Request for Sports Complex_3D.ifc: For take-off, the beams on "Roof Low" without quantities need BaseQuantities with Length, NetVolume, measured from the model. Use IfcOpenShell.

First a look at what the model holds.

```python
import ifcopenshell
import ifcopenshell.util.element
import ifcopenshell.util.unit

model = ifcopenshell.open("Sports Complex_3D.ifc")
print(model.schema)
for unit_type in ("LENGTHUNIT", "AREAUNIT", "VOLUMEUNIT"):
    print(unit_type, ifcopenshell.util.unit.calculate_unit_scale(model, unit_type))
storey = next(s for s in model.by_type("IfcBuildingStorey") if s.Name == "Roof Low")
beams = [e for e in ifcopenshell.util.element.get_decomposition(storey) if e.is_a("IfcBeam")]
for e in sorted(beams, key=lambda e: e.id()):
    print(e.id(), e.is_a(), e.Name, list(ifcopenshell.util.element.get_psets(e, qtos_only=True)), sep=" | ")
```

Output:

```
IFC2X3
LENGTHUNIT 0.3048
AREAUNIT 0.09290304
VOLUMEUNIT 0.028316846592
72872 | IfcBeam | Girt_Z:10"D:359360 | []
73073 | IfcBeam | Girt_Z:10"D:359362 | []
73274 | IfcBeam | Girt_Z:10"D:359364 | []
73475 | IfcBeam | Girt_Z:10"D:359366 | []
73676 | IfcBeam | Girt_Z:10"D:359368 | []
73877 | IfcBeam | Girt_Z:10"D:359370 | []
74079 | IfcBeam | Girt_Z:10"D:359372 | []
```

```python
import ifcopenshell
import ifcopenshell.api.pset
import ifcopenshell.geom
import ifcopenshell.util.element
import ifcopenshell.util.shape
import ifcopenshell.util.unit

model = ifcopenshell.open("Sports Complex_3D.ifc")
unit_scale = ifcopenshell.util.unit.calculate_unit_scale(model)
volume_scale = ifcopenshell.util.unit.calculate_unit_scale(model, "VOLUMEUNIT")
settings = ifcopenshell.geom.settings()

storey = next(s for s in model.by_type("IfcBuildingStorey") if s.Name == "Roof Low")
beams = [e for e in ifcopenshell.util.element.get_decomposition(storey) if e.is_a("IfcBeam")]

for e in sorted(beams, key=lambda e: e.id()):
    if ifcopenshell.util.element.get_psets(e, qtos_only=True, should_inherit=False):
        continue
    # Geometry comes back in metres, in the element's own axes.
    shape = ifcopenshell.geom.create_shape(settings, e)
    values = {
        "Length": ifcopenshell.util.shape.get_max_xyz(shape.geometry) / unit_scale,
        "NetVolume": ifcopenshell.util.shape.get_volume(shape.geometry) / volume_scale,
    }
    qto = ifcopenshell.api.pset.add_qto(model, product=e, name="BaseQuantities")
    ifcopenshell.api.pset.edit_qto(model, qto=qto, properties=values)
    print(e.id(), {k: round(v, 3) for k, v in values.items()})

model.write("Sports Complex_3D-out.ifc")
```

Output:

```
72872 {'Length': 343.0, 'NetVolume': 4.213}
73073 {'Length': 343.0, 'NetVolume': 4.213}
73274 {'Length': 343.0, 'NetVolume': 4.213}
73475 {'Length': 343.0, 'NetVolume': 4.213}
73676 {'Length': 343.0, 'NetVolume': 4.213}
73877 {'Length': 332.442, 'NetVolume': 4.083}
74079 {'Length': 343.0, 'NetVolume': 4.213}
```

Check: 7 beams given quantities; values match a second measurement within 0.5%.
